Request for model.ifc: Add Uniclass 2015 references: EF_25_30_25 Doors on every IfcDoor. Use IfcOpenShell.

First a look at what the model holds.

```python
import ifcopenshell

model = ifcopenshell.open("model.ifc")
print(model.schema)
print("classifications:", [c.Name for c in model.by_type("IfcClassification")])
for ifc_class in ("IfcDoor", "IfcRoof", "IfcStair", "IfcWall", "IfcWindow"):
    print(ifc_class, len(model.by_type(ifc_class)))
```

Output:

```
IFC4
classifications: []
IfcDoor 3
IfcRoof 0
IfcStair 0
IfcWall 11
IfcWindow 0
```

```python
import ifcopenshell
import ifcopenshell.api.classification

model = ifcopenshell.open("model.ifc")

system = ifcopenshell.api.classification.add_classification(model, classification="Uniclass 2015")

codes = {
    "IfcDoor": ("EF_25_30_25", "Doors"),
}
for ifc_class, (code, name) in codes.items():
    products = model.by_type(ifc_class)
    ifcopenshell.api.classification.add_reference(
        model, products=products, classification=system, identification=code, name=name
    )
    print(code, len(products))

model.write("model_rev.ifc")
```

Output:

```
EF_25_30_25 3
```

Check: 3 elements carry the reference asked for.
